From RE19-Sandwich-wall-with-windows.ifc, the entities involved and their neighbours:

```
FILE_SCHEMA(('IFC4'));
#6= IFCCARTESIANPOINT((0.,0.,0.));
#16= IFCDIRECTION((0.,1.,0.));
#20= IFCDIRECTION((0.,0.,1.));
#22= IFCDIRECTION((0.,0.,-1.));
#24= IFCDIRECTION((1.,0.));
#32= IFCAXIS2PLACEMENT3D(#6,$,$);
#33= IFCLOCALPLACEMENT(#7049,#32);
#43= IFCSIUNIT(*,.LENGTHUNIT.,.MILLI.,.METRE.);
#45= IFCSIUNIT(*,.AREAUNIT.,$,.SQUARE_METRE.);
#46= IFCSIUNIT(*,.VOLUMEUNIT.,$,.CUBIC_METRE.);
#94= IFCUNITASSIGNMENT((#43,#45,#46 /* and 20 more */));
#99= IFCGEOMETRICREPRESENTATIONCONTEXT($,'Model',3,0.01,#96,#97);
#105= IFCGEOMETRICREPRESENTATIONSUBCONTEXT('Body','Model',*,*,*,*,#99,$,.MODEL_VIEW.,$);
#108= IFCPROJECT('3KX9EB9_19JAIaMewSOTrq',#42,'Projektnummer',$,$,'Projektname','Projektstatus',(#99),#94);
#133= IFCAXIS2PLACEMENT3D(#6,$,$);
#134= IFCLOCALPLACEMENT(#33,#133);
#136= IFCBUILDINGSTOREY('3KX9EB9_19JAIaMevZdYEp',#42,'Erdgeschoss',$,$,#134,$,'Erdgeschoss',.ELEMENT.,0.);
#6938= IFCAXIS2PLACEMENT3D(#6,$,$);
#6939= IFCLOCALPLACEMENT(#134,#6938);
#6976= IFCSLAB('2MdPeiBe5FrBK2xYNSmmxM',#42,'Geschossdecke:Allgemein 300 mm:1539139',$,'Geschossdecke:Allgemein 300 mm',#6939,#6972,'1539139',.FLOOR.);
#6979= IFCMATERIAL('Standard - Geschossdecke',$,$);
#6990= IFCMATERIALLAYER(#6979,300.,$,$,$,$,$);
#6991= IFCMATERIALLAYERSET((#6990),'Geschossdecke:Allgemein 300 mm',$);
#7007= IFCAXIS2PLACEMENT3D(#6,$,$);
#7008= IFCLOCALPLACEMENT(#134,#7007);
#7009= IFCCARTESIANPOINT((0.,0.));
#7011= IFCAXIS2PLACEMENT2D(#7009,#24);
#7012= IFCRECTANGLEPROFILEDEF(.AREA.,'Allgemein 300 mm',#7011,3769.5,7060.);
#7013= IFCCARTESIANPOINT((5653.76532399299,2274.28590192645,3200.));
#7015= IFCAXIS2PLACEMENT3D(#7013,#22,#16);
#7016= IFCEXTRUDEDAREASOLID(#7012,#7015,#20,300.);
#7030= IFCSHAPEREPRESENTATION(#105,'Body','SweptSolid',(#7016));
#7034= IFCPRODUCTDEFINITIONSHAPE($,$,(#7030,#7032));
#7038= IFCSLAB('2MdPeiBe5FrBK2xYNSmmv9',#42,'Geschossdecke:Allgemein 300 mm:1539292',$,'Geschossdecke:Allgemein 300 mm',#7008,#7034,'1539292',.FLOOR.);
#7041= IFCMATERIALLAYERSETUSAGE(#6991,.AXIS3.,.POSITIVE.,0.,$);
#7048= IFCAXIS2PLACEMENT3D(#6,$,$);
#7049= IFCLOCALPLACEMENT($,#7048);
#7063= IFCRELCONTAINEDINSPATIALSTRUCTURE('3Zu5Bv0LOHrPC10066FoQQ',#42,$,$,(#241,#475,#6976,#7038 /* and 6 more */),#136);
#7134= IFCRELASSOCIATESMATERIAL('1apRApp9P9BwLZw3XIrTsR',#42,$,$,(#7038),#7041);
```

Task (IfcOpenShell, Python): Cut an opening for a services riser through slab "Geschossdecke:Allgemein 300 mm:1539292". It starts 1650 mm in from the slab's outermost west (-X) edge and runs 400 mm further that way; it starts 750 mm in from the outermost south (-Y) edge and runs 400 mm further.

```python
import numpy as np
import ifcopenshell
import ifcopenshell.api.feature
import ifcopenshell.api.geometry
import ifcopenshell.api.root
import ifcopenshell.geom
import ifcopenshell.util.placement
import ifcopenshell.util.representation
import ifcopenshell.util.shape
import ifcopenshell.util.unit

model = ifcopenshell.open("RE19-Sandwich-wall-with-windows.ifc")
unit_scale = ifcopenshell.util.unit.calculate_unit_scale(model)
settings = ifcopenshell.geom.settings()


def volume(element):
    """Net volume in cubic metres, openings subtracted."""
    shape = ifcopenshell.geom.create_shape(settings, element)
    return ifcopenshell.util.shape.get_volume(shape.geometry)


slab = model.by_guid("2MdPeiBe5FrBK2xYNSmmv9")
before = volume(slab)

# Extent in the slab's own axes, in metres. The edges named are its -X and -Y sides.
slab_shape = ifcopenshell.geom.create_shape(settings, slab)
vertices = ifcopenshell.util.shape.get_vertices(slab_shape.geometry)
x_min, y_min, bottom = vertices.min(axis=0)
top = vertices[:, 2].max()

opening = ifcopenshell.api.root.create_entity(model, ifc_class="IfcOpeningElement", name="Services riser opening", predefined_type="OPENING")
context = ifcopenshell.util.representation.get_context(model, "Model", "Body", "MODEL_VIEW")
width, depth = 0.4, 0.4
outline = [(0.0, 0.0), (width, 0.0), (width, depth), (0.0, depth), (0.0, 0.0)]
# Overshoot both faces by 50 mm so the cut is clean.
shape = ifcopenshell.api.geometry.add_slab_representation(
    model, context=context, depth=top - bottom + 0.1, polyline=outline
)
ifcopenshell.api.geometry.assign_representation(model, product=opening, representation=shape)

matrix = ifcopenshell.util.placement.get_local_placement(slab.ObjectPlacement)
matrix[:, 3] = matrix @ np.append(np.array([x_min + 1.65, y_min + 0.75, bottom - 0.05]) / unit_scale, 1.0)
ifcopenshell.api.geometry.edit_object_placement(model, product=opening, matrix=matrix, is_si=False)
ifcopenshell.api.feature.add_feature(model, feature=opening, element=slab)

after = volume(slab)

print(f"slab volume {before:.3f} -> {after:.3f} m3")

model.write("RE19-Sandwich-wall-with-windows_edited.ifc")
```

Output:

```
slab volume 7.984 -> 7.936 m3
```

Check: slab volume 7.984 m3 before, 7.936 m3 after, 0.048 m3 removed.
